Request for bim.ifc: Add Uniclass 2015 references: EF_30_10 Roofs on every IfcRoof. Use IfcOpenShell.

First a look at what the model holds.

```python
import ifcopenshell

model = ifcopenshell.open("bim.ifc")
print(model.schema)
print("classifications:", [c.Name for c in model.by_type("IfcClassification")])
for ifc_class in ("IfcDoor", "IfcRoof", "IfcStair", "IfcWall", "IfcWindow"):
    print(ifc_class, len(model.by_type(ifc_class)))
```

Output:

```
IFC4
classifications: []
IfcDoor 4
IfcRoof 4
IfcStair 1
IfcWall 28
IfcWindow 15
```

```python
import ifcopenshell
import ifcopenshell.api.classification

model = ifcopenshell.open("bim.ifc")

system = ifcopenshell.api.classification.add_classification(model, classification="Uniclass 2015")

codes = {
    "IfcRoof": ("EF_30_10", "Roofs"),
}
for ifc_class, (code, name) in codes.items():
    products = model.by_type(ifc_class)
    ifcopenshell.api.classification.add_reference(
        model, products=products, classification=system, identification=code, name=name
    )
    print(code, len(products))

model.write("bim_edited.ifc")
```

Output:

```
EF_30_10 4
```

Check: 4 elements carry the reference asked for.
